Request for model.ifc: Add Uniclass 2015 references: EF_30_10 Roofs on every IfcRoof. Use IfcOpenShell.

First a look at what the model holds.

```python
import ifcopenshell

model = ifcopenshell.open("model.ifc")
print(model.schema)
print("classifications:", [c.Name for c in model.by_type("IfcClassification")])
for ifc_class in ("IfcDoor", "IfcRoof", "IfcStair", "IfcWall", "IfcWindow"):
    print(ifc_class, len(model.by_type(ifc_class)))
```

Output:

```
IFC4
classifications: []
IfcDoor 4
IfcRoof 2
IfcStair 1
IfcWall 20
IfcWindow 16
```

```python
import ifcopenshell
import ifcopenshell.api.classification

model = ifcopenshell.open("model.ifc")

system = ifcopenshell.api.classification.add_classification(model, classification="Uniclass 2015")

codes = {
    "IfcRoof": ("EF_30_10", "Roofs"),
}
for ifc_class, (code, name) in codes.items():
    products = model.by_type(ifc_class)
    ifcopenshell.api.classification.add_reference(
        model, products=products, classification=system, identification=code, name=name
    )
    print(code, len(products))

model.write("model_v2.ifc")
```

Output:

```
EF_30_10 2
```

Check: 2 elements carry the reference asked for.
